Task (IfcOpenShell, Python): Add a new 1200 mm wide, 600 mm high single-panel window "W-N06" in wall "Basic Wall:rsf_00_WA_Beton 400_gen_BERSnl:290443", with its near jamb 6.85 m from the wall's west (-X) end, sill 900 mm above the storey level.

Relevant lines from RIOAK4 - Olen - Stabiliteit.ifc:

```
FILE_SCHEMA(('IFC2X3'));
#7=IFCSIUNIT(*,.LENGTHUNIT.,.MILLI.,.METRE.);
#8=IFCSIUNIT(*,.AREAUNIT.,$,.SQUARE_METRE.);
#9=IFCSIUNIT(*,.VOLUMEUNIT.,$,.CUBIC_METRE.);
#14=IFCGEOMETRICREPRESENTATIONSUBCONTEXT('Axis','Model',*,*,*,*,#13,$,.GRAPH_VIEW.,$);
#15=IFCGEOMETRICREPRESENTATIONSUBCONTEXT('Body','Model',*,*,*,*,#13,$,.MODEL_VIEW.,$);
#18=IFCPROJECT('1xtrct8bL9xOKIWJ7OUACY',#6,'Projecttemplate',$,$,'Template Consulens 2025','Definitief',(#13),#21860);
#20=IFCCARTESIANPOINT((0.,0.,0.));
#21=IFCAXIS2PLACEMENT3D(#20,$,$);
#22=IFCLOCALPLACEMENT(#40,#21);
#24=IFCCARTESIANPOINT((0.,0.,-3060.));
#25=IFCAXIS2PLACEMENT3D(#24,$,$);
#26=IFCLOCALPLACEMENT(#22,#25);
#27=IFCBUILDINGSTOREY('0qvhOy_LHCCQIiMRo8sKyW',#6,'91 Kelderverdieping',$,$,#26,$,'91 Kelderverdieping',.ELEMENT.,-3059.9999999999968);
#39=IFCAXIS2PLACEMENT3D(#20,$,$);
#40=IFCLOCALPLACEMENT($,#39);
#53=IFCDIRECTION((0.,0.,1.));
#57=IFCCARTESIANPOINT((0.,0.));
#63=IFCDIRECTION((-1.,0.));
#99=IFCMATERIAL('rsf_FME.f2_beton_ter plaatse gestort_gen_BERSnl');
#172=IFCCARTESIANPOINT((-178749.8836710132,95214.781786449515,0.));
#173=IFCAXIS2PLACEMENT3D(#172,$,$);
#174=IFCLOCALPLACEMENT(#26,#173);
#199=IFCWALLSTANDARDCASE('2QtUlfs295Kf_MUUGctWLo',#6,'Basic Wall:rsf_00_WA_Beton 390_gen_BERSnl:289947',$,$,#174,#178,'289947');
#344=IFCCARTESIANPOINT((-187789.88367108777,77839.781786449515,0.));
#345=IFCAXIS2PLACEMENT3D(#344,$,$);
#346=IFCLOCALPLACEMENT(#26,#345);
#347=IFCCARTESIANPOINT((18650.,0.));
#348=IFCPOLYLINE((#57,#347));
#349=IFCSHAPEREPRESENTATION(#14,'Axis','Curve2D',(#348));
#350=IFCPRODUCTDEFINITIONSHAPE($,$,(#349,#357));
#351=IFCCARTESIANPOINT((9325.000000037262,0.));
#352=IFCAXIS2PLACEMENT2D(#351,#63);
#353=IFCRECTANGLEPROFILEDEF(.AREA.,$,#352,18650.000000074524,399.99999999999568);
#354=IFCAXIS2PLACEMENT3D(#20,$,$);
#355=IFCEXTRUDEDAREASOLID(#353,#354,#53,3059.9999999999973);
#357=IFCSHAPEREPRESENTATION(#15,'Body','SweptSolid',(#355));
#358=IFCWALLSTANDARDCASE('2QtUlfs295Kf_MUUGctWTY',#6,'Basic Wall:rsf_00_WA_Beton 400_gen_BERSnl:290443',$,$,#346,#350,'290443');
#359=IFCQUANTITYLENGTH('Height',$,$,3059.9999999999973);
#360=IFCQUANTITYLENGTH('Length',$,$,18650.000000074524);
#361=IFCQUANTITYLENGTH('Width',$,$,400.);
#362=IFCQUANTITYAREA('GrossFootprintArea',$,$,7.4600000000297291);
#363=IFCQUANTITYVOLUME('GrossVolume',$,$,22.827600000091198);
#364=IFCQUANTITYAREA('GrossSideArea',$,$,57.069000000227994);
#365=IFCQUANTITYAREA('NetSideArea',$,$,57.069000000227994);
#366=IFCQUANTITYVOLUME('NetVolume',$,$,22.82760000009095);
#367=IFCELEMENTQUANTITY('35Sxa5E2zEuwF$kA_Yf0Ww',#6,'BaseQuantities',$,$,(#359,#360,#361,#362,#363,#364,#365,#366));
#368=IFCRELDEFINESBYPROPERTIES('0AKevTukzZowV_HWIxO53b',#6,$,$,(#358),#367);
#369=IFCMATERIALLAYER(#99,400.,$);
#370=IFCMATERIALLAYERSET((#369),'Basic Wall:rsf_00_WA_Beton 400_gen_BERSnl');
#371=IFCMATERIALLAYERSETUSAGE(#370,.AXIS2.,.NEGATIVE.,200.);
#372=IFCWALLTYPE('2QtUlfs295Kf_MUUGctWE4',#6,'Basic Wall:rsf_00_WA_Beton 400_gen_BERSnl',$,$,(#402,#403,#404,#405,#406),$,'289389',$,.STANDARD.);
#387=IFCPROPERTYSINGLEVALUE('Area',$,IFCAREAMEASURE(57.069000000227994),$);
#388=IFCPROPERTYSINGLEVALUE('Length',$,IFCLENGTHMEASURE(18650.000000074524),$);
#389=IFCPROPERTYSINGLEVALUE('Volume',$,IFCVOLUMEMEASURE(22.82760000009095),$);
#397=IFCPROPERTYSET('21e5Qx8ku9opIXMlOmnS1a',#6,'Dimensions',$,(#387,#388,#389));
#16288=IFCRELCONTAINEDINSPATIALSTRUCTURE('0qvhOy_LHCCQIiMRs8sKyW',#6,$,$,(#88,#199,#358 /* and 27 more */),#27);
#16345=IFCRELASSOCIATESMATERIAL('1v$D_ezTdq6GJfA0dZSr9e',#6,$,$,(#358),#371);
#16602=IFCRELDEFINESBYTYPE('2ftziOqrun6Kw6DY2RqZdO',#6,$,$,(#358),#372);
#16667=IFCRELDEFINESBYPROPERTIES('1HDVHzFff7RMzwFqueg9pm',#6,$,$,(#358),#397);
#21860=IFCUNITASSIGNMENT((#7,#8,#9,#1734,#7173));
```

```python
import numpy as np
import ifcopenshell
import ifcopenshell.api.feature
import ifcopenshell.api.geometry
import ifcopenshell.api.pset
import ifcopenshell.api.root
import ifcopenshell.api.spatial
import ifcopenshell.api.type
import ifcopenshell.geom
import ifcopenshell.util.element
import ifcopenshell.util.placement
import ifcopenshell.util.representation
import ifcopenshell.util.shape
import ifcopenshell.util.unit

model = ifcopenshell.open("RIOAK4 - Olen - Stabiliteit.ifc")
unit_scale = ifcopenshell.util.unit.calculate_unit_scale(model)
area_scale = ifcopenshell.util.unit.calculate_unit_scale(model, "AREAUNIT")
volume_scale = ifcopenshell.util.unit.calculate_unit_scale(model, "VOLUMEUNIT")
settings = ifcopenshell.geom.settings()


def volume(element):
    """Net volume in cubic metres, openings subtracted."""
    shape = ifcopenshell.geom.create_shape(settings, element)
    return ifcopenshell.util.shape.get_volume(shape.geometry)


wall = model.by_guid("2QtUlfs295Kf_MUUGctWTY")
storey = ifcopenshell.util.element.get_container(wall, ifc_class="IfcBuildingStorey")
context = ifcopenshell.util.representation.get_context(model, "Model", "Body", "MODEL_VIEW")
before = volume(wall)

width, height, from_end, sill = 1.2, 0.6, 6.85, 0.9  # metres

# The wall runs along its own X axis, and the end named is its -X end.
wall_shape = ifcopenshell.geom.create_shape(settings, wall)
x, y, z = ifcopenshell.util.shape.get_vertices(wall_shape.geometry).T
start = x.min() + from_end
face, thickness = float(y.min()), float(y.max() - y.min())
wall_matrix = ifcopenshell.util.placement.get_local_placement(wall.ObjectPlacement)
level = ifcopenshell.util.placement.get_local_placement(storey.ObjectPlacement)[2, 3]


def in_wall(x, y):
    """Placement at x, y metres in the wall's axes, at sill height."""
    matrix = wall_matrix.copy()
    matrix[:, 3] = wall_matrix @ np.array([x / unit_scale, y / unit_scale, 0.0, 1.0])
    matrix[2, 3] = level + sill / unit_scale
    return matrix


# Opening: a box that overshoots both wall faces by 50 mm.
opening = ifcopenshell.api.root.create_entity(model, ifc_class="IfcOpeningElement")
box = ifcopenshell.api.geometry.add_wall_representation(
    model, context=context, length=width, height=height, thickness=thickness + 0.1
)
ifcopenshell.api.geometry.assign_representation(model, product=opening, representation=box)
ifcopenshell.api.geometry.edit_object_placement(model, product=opening, matrix=in_wall(start, face - 0.05), is_si=False)
ifcopenshell.api.feature.add_feature(model, feature=opening, element=wall)

window = ifcopenshell.api.root.create_entity(model, ifc_class="IfcWindow", name="W-N06")
window.OverallWidth, window.OverallHeight = width / unit_scale, height / unit_scale
body = ifcopenshell.api.geometry.add_window_representation(
    model,
    context=context,
    overall_width=window.OverallWidth,
    overall_height=window.OverallHeight,
    partition_type="SINGLE_PANEL",
)
ifcopenshell.api.geometry.assign_representation(model, product=window, representation=body)
ifcopenshell.api.spatial.assign_container(model, products=[window], relating_structure=storey)
fills = ifcopenshell.api.feature.add_filling(model, opening=opening, element=window)
fills.OwnerHistory = window.OwnerHistory  # required in IFC2X3

# IFC2X3 keeps the operation on the window style.
style = ifcopenshell.api.root.create_entity(model, ifc_class="IfcWindowStyle", name="W-N06")
style.OperationType, style.ConstructionType = "SINGLE_PANEL", "NOTDEFINED"
style.ParameterTakesPrecedence = style.Sizeable = False
ifcopenshell.api.type.assign_type(model, related_objects=[window], relating_type=style)

# Centre the window in the wall's thickness.
ifcopenshell.api.geometry.edit_object_placement(model, product=window, matrix=in_wall(start, face), is_si=False)
window_shape = ifcopenshell.geom.create_shape(settings, window)
depth = ifcopenshell.util.shape.get_vertices(window_shape.geometry)[:, 1]
offset = face + thickness / 2 - (depth.min() + depth.max()) / 2
ifcopenshell.api.geometry.edit_object_placement(model, product=window, matrix=in_wall(start, offset), is_si=False)

after = volume(wall)

# Update the wall's stored quantities.
qto = model.by_id(ifcopenshell.util.element.get_pset(wall, "BaseQuantities", should_inherit=False)["id"])
ifcopenshell.api.pset.edit_qto(model, qto=qto, properties={
    "NetSideArea": after / thickness / area_scale,
    "NetVolume": after / volume_scale,
})
pset = model.by_id(ifcopenshell.util.element.get_pset(wall, "Dimensions", should_inherit=False)["id"])
ifcopenshell.api.pset.edit_pset(model, pset=pset, properties={
    "Area": model.create_entity("IfcAreaMeasure", after / thickness / area_scale),
    "Volume": model.create_entity("IfcVolumeMeasure", after / volume_scale),
})

print(f"wall volume {before:.3f} -> {after:.3f} m3")

model.write("RIOAK4 - Olen - Stabiliteit_v2.ifc")
```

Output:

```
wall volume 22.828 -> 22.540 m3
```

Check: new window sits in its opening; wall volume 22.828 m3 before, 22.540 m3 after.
